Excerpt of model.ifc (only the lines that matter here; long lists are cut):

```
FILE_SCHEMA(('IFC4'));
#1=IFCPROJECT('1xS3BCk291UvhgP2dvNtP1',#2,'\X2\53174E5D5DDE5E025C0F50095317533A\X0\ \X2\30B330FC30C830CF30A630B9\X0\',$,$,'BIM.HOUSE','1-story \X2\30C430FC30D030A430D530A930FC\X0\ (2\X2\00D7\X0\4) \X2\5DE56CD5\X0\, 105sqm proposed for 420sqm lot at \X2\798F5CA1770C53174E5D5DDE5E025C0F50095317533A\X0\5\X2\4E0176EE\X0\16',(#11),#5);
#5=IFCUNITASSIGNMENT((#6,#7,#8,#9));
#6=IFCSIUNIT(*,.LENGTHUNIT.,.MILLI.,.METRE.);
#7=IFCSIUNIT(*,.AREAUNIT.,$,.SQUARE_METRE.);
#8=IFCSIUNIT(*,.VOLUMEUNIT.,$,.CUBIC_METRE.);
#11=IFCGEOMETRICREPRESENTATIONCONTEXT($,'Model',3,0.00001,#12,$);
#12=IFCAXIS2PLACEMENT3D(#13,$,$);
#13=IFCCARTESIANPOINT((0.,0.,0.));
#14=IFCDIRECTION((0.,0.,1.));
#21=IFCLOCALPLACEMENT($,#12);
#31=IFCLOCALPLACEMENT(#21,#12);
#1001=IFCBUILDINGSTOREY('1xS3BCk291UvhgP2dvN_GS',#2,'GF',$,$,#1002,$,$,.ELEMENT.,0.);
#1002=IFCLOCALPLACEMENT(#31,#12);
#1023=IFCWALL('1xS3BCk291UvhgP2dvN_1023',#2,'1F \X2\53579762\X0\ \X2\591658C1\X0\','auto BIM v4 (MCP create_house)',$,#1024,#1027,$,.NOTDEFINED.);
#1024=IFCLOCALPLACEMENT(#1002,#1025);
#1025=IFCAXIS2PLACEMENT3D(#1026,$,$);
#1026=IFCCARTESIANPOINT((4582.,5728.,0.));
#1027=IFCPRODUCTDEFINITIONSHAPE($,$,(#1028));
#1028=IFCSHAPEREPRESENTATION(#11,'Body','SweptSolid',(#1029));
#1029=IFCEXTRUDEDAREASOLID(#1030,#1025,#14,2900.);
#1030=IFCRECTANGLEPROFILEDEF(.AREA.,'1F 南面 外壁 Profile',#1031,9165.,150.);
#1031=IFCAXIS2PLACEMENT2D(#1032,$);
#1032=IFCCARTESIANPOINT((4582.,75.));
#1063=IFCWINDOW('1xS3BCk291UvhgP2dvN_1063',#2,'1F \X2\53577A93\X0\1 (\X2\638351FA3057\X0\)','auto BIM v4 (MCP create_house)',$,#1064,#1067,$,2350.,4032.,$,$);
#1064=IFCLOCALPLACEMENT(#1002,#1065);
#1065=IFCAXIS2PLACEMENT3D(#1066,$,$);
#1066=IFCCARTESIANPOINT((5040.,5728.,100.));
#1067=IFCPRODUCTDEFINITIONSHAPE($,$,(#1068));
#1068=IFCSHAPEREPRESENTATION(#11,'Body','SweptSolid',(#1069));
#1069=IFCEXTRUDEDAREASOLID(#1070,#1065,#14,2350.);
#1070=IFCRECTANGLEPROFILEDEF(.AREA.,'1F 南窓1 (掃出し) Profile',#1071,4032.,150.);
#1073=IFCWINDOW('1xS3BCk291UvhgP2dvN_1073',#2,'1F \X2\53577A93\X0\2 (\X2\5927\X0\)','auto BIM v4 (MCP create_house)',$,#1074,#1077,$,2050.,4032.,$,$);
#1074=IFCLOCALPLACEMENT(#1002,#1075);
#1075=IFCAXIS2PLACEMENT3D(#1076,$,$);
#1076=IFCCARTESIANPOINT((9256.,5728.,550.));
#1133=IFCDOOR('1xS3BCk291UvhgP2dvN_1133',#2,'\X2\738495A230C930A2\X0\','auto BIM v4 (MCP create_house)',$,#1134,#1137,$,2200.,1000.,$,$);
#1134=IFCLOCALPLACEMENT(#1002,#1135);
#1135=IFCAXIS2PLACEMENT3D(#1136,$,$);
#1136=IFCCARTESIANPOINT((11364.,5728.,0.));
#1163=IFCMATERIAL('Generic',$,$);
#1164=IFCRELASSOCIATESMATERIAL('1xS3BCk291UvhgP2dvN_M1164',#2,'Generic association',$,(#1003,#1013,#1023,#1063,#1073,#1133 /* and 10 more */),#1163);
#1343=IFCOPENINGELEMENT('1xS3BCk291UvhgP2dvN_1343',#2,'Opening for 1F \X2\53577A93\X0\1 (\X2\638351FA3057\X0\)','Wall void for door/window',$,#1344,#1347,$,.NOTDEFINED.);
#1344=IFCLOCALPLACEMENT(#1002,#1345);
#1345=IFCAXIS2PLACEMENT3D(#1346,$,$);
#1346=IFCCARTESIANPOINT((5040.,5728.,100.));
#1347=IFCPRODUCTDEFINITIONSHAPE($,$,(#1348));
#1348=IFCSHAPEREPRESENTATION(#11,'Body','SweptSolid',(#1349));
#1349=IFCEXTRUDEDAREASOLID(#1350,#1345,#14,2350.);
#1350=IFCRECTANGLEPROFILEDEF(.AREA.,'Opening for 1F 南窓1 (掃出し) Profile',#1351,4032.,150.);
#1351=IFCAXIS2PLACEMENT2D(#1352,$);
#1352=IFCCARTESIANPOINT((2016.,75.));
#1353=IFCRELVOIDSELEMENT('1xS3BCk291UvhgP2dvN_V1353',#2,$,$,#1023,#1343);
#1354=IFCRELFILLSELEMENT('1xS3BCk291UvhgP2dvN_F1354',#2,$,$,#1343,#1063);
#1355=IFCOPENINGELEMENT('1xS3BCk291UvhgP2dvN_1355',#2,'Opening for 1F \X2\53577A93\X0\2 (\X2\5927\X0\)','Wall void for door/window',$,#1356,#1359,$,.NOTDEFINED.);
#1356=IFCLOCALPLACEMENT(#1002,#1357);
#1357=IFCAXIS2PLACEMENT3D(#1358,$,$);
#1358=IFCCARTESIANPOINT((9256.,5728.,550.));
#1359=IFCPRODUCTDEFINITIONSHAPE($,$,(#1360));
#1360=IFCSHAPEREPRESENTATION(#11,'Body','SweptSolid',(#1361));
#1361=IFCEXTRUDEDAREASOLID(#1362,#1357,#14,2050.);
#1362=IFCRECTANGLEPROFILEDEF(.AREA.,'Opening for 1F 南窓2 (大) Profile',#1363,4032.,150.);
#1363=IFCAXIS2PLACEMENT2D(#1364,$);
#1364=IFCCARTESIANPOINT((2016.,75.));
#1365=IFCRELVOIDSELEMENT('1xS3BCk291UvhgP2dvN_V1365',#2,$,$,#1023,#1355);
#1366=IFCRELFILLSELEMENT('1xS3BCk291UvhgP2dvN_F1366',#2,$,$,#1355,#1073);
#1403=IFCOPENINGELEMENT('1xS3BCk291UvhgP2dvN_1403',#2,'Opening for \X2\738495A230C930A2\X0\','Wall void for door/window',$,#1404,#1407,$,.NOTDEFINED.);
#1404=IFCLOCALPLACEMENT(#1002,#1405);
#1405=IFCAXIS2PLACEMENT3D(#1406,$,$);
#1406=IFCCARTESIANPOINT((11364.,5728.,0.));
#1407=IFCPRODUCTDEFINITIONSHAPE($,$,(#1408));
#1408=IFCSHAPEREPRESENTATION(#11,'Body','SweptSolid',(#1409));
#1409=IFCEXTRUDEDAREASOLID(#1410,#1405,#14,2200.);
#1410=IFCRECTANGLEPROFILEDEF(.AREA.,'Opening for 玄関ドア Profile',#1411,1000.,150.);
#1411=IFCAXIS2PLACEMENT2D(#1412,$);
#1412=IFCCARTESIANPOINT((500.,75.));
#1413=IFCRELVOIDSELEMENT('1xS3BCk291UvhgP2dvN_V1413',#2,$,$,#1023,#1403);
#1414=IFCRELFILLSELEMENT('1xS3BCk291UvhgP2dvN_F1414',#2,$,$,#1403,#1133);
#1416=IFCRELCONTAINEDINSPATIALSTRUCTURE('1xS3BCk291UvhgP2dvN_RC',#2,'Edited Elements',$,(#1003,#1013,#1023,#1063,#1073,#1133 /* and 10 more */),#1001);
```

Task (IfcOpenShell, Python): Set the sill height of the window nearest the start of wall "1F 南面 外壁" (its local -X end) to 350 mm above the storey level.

```python
import numpy as np
import ifcopenshell
import ifcopenshell.api.geometry
import ifcopenshell.geom
import ifcopenshell.util.element
import ifcopenshell.util.placement
import ifcopenshell.util.shape
import ifcopenshell.util.unit

model = ifcopenshell.open("model.ifc")
unit_scale = ifcopenshell.util.unit.calculate_unit_scale(model)

window = model.by_guid("1xS3BCk291UvhgP2dvN_1063")
opening = window.FillsVoids[0].RelatingOpeningElement
storey = ifcopenshell.util.element.get_container(window, ifc_class="IfcBuildingStorey")
level = ifcopenshell.util.placement.get_local_placement(storey.ObjectPlacement)[2, 3]

# The opening's origin need not be at the sill, so measure its lowest point.
shape = ifcopenshell.geom.create_shape(ifcopenshell.geom.settings(), opening)
bottom = ifcopenshell.util.shape.get_shape_bottom_elevation(shape, shape.geometry) / unit_scale
dz = level + 0.35 / unit_scale - bottom

shift = np.array([0.0, 0.0, dz])
# The window is not placed relative to its opening, so move both.
for product in (opening, window):
    matrix = ifcopenshell.util.placement.get_local_placement(product.ObjectPlacement)
    matrix[:3, 3] += shift
    ifcopenshell.api.geometry.edit_object_placement(model, product=product, matrix=matrix, is_si=False)

print(f"moved by {dz * unit_scale:+.3f} m")

model.write("model_edited.ifc")
```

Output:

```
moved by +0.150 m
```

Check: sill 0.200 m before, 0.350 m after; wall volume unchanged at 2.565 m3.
